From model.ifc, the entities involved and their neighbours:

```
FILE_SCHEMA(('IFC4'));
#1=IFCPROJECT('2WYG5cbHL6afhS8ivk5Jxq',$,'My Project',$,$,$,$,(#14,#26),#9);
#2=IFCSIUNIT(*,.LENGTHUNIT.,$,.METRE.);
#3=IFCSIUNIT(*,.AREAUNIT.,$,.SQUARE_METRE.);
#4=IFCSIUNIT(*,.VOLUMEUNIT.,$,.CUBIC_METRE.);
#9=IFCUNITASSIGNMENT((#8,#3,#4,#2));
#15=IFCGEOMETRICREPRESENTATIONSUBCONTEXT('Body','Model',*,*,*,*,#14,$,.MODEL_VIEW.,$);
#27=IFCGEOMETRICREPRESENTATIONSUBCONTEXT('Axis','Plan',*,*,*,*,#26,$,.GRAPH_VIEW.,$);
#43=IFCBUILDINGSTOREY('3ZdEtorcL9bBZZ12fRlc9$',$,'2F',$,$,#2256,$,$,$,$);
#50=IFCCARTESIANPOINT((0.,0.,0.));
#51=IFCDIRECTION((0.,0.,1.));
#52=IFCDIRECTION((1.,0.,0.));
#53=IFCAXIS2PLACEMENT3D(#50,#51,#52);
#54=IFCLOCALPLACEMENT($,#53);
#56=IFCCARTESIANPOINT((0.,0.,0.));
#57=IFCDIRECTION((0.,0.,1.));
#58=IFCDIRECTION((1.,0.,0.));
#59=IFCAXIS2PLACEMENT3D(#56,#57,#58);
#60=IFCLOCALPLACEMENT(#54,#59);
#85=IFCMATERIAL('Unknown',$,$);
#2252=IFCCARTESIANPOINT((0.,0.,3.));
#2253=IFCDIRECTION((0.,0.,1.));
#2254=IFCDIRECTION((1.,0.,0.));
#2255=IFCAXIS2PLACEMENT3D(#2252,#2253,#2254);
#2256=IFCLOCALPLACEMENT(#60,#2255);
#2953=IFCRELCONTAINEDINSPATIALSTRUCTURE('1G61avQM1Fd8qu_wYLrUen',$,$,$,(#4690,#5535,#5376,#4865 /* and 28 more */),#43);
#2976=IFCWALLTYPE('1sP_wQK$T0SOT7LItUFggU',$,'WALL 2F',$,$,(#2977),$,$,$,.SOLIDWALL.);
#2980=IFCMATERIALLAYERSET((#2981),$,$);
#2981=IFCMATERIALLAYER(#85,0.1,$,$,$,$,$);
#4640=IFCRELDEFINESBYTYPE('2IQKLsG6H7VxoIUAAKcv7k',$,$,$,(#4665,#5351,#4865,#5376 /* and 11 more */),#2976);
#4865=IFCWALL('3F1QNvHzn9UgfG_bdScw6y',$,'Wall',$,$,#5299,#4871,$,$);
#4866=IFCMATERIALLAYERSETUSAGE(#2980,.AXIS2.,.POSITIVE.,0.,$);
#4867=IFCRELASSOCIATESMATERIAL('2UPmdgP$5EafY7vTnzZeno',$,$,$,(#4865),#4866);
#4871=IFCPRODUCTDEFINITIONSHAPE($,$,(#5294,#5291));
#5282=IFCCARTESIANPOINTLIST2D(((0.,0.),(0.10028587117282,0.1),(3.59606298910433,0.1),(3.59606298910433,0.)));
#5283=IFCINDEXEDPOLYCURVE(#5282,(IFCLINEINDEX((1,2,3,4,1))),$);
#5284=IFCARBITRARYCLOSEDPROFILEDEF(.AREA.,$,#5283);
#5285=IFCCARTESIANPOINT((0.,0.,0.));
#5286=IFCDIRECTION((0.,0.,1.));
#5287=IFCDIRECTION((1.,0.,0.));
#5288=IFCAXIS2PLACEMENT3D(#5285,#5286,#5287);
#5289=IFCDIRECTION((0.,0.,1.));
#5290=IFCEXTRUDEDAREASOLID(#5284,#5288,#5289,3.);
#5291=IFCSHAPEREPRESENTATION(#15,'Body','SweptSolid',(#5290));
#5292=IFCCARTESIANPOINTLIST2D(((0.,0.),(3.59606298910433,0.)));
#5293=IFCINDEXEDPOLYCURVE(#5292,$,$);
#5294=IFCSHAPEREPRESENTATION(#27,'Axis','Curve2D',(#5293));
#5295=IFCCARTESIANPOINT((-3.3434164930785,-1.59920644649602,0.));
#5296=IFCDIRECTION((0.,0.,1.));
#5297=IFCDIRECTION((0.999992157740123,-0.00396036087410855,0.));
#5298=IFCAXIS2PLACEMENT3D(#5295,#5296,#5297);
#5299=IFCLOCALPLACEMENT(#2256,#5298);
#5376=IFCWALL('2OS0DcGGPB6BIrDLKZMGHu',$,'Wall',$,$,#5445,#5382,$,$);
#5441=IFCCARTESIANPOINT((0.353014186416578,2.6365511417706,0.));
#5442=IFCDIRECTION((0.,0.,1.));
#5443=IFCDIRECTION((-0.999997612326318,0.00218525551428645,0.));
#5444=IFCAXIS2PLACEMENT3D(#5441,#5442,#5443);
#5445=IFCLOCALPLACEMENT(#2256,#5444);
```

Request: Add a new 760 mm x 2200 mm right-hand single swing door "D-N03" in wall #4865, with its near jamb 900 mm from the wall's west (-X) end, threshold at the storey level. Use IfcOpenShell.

```python
import numpy as np
import ifcopenshell
import ifcopenshell.api.feature
import ifcopenshell.api.geometry
import ifcopenshell.api.root
import ifcopenshell.api.spatial
import ifcopenshell.geom
import ifcopenshell.util.element
import ifcopenshell.util.placement
import ifcopenshell.util.representation
import ifcopenshell.util.shape
import ifcopenshell.util.unit

model = ifcopenshell.open("model.ifc")
unit_scale = ifcopenshell.util.unit.calculate_unit_scale(model)
settings = ifcopenshell.geom.settings()


def volume(element):
    """Net volume in cubic metres, openings subtracted."""
    shape = ifcopenshell.geom.create_shape(settings, element)
    return ifcopenshell.util.shape.get_volume(shape.geometry)


wall = model.by_guid("3F1QNvHzn9UgfG_bdScw6y")
storey = ifcopenshell.util.element.get_container(wall, ifc_class="IfcBuildingStorey")
context = ifcopenshell.util.representation.get_context(model, "Model", "Body", "MODEL_VIEW")
before = volume(wall)

width, height, from_end, sill = 0.76, 2.2, 0.9, 0.0  # metres

# The wall runs along its own X axis, and the end named is its -X end.
wall_shape = ifcopenshell.geom.create_shape(settings, wall)
x, y, z = ifcopenshell.util.shape.get_vertices(wall_shape.geometry).T
start = x.min() + from_end
face, thickness = float(y.min()), float(y.max() - y.min())
wall_matrix = ifcopenshell.util.placement.get_local_placement(wall.ObjectPlacement)
level = ifcopenshell.util.placement.get_local_placement(storey.ObjectPlacement)[2, 3]


def in_wall(x, y):
    """Placement at x, y metres in the wall's axes, at sill height."""
    matrix = wall_matrix.copy()
    matrix[:, 3] = wall_matrix @ np.array([x / unit_scale, y / unit_scale, 0.0, 1.0])
    matrix[2, 3] = level + sill / unit_scale
    return matrix


# Opening: a box that overshoots both wall faces by 50 mm.
opening = ifcopenshell.api.root.create_entity(model, ifc_class="IfcOpeningElement", predefined_type="OPENING")
box = ifcopenshell.api.geometry.add_wall_representation(
    model, context=context, length=width, height=height, thickness=thickness + 0.1
)
ifcopenshell.api.geometry.assign_representation(model, product=opening, representation=box)
ifcopenshell.api.geometry.edit_object_placement(model, product=opening, matrix=in_wall(start, face - 0.05), is_si=False)
ifcopenshell.api.feature.add_feature(model, feature=opening, element=wall)

door = ifcopenshell.api.root.create_entity(model, ifc_class="IfcDoor", name="D-N03", predefined_type="DOOR")
door.OverallWidth, door.OverallHeight = width / unit_scale, height / unit_scale
door.OperationType = "SINGLE_SWING_RIGHT"
body = ifcopenshell.api.geometry.add_door_representation(
    model,
    context=context,
    overall_width=door.OverallWidth,
    overall_height=door.OverallHeight,
    operation_type="SINGLE_SWING_RIGHT",
    lining_properties={"LiningDepth": thickness / unit_scale, "ThresholdDepth": thickness / unit_scale},
)
ifcopenshell.api.geometry.assign_representation(model, product=door, representation=body)
ifcopenshell.api.spatial.assign_container(model, products=[door], relating_structure=storey)
ifcopenshell.api.feature.add_filling(model, opening=opening, element=door)

# The lining spans the wall, so the door starts at the wall face.
ifcopenshell.api.geometry.edit_object_placement(model, product=door, matrix=in_wall(start, face), is_si=False)

after = volume(wall)

print(f"wall volume {before:.3f} -> {after:.3f} m3")

model.write("model_updated.ifc")
```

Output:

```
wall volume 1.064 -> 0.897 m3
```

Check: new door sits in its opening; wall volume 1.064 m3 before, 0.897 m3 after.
